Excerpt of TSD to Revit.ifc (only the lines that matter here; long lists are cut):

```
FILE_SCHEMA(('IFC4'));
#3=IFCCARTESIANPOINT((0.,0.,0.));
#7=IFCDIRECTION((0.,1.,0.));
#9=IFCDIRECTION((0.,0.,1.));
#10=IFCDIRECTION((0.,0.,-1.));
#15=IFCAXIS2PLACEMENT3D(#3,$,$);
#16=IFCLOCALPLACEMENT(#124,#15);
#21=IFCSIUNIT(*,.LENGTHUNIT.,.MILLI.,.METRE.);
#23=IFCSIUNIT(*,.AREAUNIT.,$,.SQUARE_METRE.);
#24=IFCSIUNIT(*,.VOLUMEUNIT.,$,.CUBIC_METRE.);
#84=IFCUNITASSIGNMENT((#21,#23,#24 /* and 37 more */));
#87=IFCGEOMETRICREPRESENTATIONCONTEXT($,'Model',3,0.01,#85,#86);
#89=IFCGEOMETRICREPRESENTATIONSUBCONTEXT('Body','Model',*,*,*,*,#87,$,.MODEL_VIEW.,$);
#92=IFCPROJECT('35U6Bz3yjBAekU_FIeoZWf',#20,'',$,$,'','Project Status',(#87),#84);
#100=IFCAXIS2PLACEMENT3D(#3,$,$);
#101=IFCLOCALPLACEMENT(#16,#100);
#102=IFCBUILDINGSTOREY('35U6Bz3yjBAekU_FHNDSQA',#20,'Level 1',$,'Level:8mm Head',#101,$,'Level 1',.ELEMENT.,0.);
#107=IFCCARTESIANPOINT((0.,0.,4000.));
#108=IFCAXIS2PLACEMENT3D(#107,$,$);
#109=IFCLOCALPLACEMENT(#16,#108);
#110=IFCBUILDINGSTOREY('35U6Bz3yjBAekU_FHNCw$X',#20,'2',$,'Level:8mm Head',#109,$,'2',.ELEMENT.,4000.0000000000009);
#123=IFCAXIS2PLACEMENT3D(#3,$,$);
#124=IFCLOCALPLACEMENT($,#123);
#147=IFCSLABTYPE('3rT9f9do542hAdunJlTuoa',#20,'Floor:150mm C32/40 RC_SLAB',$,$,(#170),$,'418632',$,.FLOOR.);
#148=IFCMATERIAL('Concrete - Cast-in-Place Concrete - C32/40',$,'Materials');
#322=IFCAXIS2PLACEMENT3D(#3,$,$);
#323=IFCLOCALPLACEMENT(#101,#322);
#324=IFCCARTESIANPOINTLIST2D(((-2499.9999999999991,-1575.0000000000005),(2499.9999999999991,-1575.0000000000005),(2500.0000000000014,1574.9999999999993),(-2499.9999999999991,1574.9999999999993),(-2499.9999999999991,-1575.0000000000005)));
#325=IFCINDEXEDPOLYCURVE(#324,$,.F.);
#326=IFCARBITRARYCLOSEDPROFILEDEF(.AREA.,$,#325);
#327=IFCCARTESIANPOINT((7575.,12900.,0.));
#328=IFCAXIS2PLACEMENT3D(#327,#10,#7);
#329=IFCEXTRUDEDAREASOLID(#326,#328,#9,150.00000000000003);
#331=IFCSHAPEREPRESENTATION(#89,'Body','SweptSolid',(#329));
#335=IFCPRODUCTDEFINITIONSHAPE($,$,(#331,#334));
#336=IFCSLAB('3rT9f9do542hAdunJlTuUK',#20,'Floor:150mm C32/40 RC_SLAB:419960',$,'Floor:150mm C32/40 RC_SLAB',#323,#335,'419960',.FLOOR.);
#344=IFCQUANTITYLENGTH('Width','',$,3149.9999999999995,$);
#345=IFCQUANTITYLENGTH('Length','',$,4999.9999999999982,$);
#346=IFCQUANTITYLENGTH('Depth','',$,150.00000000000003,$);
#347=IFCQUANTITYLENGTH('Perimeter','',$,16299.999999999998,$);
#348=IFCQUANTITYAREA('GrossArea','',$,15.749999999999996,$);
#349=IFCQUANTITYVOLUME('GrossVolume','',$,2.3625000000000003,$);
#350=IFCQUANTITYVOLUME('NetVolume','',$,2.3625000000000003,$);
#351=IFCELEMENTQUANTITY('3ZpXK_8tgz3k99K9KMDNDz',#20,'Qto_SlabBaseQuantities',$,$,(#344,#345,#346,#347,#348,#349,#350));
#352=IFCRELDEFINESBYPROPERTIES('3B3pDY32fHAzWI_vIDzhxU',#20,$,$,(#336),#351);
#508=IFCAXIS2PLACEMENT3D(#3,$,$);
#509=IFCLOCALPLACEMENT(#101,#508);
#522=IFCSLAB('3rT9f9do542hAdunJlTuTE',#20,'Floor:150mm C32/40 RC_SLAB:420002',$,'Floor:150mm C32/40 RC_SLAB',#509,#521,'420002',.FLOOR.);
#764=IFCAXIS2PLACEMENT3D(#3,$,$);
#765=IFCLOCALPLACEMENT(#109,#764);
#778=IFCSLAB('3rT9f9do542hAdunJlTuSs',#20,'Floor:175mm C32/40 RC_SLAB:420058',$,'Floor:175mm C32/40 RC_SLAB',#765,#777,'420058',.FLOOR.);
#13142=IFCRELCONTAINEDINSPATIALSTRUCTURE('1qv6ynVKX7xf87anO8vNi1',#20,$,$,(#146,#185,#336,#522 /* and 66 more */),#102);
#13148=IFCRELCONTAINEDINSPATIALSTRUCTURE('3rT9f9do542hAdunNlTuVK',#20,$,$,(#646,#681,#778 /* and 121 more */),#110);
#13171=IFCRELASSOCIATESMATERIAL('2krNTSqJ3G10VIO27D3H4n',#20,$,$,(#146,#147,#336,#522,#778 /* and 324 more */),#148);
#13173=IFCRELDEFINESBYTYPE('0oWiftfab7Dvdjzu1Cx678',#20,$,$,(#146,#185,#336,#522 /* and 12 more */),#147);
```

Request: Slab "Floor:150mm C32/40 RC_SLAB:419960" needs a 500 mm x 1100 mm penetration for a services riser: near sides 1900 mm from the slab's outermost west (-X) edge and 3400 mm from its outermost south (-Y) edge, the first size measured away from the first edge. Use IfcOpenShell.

```python
import numpy as np
import ifcopenshell
import ifcopenshell.api.feature
import ifcopenshell.api.geometry
import ifcopenshell.api.pset
import ifcopenshell.api.root
import ifcopenshell.geom
import ifcopenshell.util.element
import ifcopenshell.util.placement
import ifcopenshell.util.representation
import ifcopenshell.util.shape
import ifcopenshell.util.unit

model = ifcopenshell.open("TSD to Revit.ifc")
unit_scale = ifcopenshell.util.unit.calculate_unit_scale(model)
volume_scale = ifcopenshell.util.unit.calculate_unit_scale(model, "VOLUMEUNIT")
settings = ifcopenshell.geom.settings()


def volume(element):
    """Net volume in cubic metres, openings subtracted."""
    shape = ifcopenshell.geom.create_shape(settings, element)
    return ifcopenshell.util.shape.get_volume(shape.geometry)


slab = model.by_guid("3rT9f9do542hAdunJlTuUK")
before = volume(slab)

# Extent in the slab's own axes, in metres. The edges named are its -X and -Y sides.
slab_shape = ifcopenshell.geom.create_shape(settings, slab)
vertices = ifcopenshell.util.shape.get_vertices(slab_shape.geometry)
x_min, y_min, bottom = vertices.min(axis=0)
top = vertices[:, 2].max()

opening = ifcopenshell.api.root.create_entity(model, ifc_class="IfcOpeningElement", name="Services riser opening", predefined_type="OPENING")
context = ifcopenshell.util.representation.get_context(model, "Model", "Body", "MODEL_VIEW")
width, depth = 0.5, 1.1
outline = [(0.0, 0.0), (width, 0.0), (width, depth), (0.0, depth), (0.0, 0.0)]
# Overshoot both faces by 50 mm so the cut is clean.
shape = ifcopenshell.api.geometry.add_slab_representation(
    model, context=context, depth=top - bottom + 0.1, polyline=outline
)
ifcopenshell.api.geometry.assign_representation(model, product=opening, representation=shape)

matrix = ifcopenshell.util.placement.get_local_placement(slab.ObjectPlacement)
matrix[:, 3] = matrix @ np.append(np.array([x_min + 1.9, y_min + 3.4, bottom - 0.05]) / unit_scale, 1.0)
ifcopenshell.api.geometry.edit_object_placement(model, product=opening, matrix=matrix, is_si=False)
ifcopenshell.api.feature.add_feature(model, feature=opening, element=slab)

after = volume(slab)

# Update the slab's stored quantities.
qto = model.by_id(ifcopenshell.util.element.get_pset(slab, "Qto_SlabBaseQuantities", should_inherit=False)["id"])
ifcopenshell.api.pset.edit_qto(model, qto=qto, properties={"NetVolume": after / volume_scale})

print(f"slab volume {before:.3f} -> {after:.3f} m3")

model.write("TSD to Revit_rev.ifc")
```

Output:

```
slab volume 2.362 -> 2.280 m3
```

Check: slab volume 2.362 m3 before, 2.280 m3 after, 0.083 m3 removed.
